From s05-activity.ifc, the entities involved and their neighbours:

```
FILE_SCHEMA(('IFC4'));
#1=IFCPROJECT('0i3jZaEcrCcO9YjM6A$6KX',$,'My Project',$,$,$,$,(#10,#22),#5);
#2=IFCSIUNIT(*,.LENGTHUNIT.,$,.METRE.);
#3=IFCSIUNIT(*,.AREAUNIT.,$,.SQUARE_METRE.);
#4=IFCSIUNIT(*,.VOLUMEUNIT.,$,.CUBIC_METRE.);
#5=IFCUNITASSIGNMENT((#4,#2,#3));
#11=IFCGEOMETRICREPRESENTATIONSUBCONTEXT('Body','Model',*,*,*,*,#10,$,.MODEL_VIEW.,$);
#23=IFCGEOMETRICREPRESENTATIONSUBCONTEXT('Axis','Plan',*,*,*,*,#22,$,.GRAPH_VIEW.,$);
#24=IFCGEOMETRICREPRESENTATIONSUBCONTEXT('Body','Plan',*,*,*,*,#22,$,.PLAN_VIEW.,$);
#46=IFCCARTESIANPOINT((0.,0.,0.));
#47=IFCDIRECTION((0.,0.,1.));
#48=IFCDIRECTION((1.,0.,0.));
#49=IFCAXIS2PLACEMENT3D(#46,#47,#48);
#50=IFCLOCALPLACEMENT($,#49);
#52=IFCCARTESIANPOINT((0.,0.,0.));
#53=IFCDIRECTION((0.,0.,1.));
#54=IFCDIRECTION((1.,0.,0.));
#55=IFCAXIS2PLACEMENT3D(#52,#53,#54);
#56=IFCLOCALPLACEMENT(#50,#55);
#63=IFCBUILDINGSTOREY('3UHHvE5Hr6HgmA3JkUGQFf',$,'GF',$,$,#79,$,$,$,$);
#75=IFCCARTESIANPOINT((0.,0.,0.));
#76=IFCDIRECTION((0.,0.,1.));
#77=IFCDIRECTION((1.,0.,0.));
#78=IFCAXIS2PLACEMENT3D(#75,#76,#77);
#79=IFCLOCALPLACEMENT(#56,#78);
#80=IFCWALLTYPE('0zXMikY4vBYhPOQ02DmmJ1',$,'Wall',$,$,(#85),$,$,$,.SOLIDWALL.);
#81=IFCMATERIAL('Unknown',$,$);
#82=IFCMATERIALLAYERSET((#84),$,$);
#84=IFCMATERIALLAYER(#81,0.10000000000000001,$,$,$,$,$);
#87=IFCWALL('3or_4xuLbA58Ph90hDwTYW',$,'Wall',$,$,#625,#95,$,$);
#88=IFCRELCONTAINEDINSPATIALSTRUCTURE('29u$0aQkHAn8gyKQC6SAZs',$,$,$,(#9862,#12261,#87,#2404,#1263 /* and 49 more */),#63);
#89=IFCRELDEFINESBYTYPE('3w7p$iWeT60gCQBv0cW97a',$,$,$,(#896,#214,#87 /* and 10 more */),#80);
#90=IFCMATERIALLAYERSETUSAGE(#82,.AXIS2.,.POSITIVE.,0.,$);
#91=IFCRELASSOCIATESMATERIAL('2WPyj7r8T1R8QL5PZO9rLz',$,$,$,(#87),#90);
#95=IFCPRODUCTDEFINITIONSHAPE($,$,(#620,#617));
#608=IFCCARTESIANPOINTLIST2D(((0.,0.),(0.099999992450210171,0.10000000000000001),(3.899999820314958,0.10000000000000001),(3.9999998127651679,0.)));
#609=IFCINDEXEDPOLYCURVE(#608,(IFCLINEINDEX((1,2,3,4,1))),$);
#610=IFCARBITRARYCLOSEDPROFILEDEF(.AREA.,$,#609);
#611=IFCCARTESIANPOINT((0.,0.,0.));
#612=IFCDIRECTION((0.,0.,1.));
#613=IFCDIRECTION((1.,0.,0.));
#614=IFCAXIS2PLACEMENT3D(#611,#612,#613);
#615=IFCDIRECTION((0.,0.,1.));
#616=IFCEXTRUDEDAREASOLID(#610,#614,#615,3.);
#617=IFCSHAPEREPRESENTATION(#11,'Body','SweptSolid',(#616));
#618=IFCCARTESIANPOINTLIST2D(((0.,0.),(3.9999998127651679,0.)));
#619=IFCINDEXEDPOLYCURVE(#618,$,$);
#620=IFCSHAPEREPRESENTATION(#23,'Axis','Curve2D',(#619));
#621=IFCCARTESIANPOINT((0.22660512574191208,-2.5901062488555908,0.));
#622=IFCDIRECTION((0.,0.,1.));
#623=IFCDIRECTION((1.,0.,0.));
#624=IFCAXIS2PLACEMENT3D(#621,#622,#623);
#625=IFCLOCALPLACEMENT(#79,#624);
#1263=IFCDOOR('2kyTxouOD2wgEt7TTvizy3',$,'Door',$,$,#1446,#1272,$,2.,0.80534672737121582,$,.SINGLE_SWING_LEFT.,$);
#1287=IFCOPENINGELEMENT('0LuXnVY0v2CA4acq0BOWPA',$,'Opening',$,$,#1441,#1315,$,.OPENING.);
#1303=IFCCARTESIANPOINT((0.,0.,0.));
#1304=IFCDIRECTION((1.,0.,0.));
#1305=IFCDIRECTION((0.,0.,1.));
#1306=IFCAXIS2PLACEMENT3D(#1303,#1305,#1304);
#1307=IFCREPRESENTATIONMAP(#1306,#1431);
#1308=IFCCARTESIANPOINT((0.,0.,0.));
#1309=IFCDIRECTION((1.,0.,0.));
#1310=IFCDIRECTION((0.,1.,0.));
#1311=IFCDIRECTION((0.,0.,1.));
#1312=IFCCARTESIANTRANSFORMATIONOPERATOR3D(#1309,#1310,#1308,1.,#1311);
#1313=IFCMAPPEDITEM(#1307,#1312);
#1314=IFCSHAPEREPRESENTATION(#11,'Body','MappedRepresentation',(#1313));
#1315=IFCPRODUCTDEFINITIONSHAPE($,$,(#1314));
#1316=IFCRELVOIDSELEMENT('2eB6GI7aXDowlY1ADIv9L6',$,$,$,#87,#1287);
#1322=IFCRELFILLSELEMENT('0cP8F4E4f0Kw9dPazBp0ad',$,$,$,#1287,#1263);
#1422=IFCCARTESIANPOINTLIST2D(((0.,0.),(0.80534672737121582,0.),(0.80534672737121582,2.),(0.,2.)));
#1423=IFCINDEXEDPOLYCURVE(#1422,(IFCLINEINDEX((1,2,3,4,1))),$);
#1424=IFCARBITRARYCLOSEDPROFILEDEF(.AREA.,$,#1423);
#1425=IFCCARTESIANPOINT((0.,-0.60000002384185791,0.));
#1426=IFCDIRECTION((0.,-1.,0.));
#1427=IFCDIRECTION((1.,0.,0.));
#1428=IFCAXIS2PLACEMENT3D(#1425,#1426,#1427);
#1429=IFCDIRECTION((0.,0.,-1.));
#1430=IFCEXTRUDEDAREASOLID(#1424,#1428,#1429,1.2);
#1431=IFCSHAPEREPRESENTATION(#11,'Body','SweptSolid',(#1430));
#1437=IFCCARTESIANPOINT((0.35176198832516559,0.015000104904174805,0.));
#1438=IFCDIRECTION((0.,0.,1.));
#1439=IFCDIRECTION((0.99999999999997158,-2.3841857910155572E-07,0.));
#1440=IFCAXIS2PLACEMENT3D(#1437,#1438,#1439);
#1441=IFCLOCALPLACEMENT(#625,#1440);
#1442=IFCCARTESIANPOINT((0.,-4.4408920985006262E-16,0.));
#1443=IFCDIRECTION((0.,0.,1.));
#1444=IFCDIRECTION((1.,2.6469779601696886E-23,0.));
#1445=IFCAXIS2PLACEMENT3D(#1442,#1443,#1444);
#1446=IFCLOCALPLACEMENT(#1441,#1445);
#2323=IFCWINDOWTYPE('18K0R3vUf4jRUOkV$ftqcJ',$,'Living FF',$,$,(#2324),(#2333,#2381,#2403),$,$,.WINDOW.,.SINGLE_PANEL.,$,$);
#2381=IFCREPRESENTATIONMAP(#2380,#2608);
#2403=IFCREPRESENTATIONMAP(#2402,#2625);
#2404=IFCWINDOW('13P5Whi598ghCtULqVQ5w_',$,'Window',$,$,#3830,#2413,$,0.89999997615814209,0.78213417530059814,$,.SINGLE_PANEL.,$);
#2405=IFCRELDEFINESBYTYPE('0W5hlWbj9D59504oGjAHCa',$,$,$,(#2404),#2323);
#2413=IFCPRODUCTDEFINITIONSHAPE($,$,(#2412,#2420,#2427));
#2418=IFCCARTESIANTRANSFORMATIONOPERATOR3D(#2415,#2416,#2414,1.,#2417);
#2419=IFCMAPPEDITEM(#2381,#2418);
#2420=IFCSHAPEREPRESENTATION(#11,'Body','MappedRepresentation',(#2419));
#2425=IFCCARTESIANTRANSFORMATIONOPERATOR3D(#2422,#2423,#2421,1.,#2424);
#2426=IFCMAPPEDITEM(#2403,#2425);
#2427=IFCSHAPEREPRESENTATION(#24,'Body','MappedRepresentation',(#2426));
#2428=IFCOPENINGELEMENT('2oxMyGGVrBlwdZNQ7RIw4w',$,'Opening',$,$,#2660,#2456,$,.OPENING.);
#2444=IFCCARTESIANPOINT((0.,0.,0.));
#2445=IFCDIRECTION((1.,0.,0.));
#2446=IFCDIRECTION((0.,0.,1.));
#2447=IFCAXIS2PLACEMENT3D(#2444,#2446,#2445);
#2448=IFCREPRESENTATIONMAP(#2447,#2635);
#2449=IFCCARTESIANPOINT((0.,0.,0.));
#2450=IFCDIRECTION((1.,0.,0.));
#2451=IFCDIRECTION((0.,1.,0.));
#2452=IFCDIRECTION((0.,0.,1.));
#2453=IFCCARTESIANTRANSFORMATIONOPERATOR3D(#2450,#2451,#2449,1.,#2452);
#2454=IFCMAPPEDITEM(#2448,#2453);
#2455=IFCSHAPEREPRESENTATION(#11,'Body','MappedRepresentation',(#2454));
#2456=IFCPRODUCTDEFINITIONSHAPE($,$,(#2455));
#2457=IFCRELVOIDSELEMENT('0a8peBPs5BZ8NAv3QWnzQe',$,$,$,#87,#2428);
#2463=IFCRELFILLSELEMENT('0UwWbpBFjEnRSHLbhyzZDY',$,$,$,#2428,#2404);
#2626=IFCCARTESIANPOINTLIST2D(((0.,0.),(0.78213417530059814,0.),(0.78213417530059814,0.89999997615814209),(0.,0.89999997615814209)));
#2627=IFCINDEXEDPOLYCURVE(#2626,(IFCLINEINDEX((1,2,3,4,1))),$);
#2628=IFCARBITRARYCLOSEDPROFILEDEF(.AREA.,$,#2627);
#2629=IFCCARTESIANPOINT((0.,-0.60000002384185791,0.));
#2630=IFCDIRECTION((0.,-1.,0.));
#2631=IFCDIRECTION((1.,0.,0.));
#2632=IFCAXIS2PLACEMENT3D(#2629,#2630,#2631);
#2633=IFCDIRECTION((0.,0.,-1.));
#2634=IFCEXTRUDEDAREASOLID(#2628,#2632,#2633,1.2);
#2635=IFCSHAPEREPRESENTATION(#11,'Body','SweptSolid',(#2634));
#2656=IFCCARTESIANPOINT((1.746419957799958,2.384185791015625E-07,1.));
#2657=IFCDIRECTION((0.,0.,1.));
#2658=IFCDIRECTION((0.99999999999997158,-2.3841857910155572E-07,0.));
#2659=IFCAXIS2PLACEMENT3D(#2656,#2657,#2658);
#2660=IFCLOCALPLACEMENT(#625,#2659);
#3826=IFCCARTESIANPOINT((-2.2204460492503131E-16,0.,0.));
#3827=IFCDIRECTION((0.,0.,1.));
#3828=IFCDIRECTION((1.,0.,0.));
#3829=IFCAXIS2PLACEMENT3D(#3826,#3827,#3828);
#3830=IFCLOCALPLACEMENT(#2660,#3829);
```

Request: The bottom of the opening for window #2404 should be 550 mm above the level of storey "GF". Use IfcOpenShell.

```python
import numpy as np
import ifcopenshell
import ifcopenshell.api.geometry
import ifcopenshell.geom
import ifcopenshell.util.element
import ifcopenshell.util.placement
import ifcopenshell.util.shape
import ifcopenshell.util.unit

model = ifcopenshell.open("s05-activity.ifc")
unit_scale = ifcopenshell.util.unit.calculate_unit_scale(model)

window = model.by_guid("13P5Whi598ghCtULqVQ5w_")
opening = window.FillsVoids[0].RelatingOpeningElement
storey = ifcopenshell.util.element.get_container(window, ifc_class="IfcBuildingStorey")
level = ifcopenshell.util.placement.get_local_placement(storey.ObjectPlacement)[2, 3]

# The opening's origin need not be at the sill, so measure its lowest point.
shape = ifcopenshell.geom.create_shape(ifcopenshell.geom.settings(), opening)
bottom = ifcopenshell.util.shape.get_shape_bottom_elevation(shape, shape.geometry) / unit_scale
dz = level + 0.55 - bottom

shift = np.array([0.0, 0.0, dz])
# The window is placed relative to its opening, so it follows when the opening moves.
matrix = ifcopenshell.util.placement.get_local_placement(opening.ObjectPlacement)
matrix[:3, 3] += shift
ifcopenshell.api.geometry.edit_object_placement(
    model, product=opening, matrix=matrix, is_si=False, should_transform_children=True
)

print(f"moved by {dz * unit_scale:+.3f} m")

model.write("s05-activity_edited.ifc")
```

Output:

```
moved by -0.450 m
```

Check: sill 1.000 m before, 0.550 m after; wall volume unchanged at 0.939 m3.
